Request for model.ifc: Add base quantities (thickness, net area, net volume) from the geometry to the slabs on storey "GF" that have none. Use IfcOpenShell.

First a look at what the model holds.

```python
import ifcopenshell
import ifcopenshell.util.element
import ifcopenshell.util.unit

model = ifcopenshell.open("model.ifc")
print(model.schema)
for unit_type in ("LENGTHUNIT", "AREAUNIT", "VOLUMEUNIT"):
    print(unit_type, ifcopenshell.util.unit.calculate_unit_scale(model, unit_type))
storey = next(s for s in model.by_type("IfcBuildingStorey") if s.Name == "GF")
slabs = [e for e in ifcopenshell.util.element.get_decomposition(storey) if e.is_a("IfcSlab")]
for e in sorted(slabs, key=lambda e: e.id()):
    print(e.id(), e.is_a(), e.Name, list(ifcopenshell.util.element.get_psets(e, qtos_only=True)), sep=" | ")
```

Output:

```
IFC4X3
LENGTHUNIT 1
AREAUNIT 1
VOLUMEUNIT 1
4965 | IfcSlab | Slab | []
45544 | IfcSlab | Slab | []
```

```python
import ifcopenshell
import ifcopenshell.api.pset
import ifcopenshell.geom
import ifcopenshell.util.element
import ifcopenshell.util.shape
import ifcopenshell.util.unit

model = ifcopenshell.open("model.ifc")
unit_scale = ifcopenshell.util.unit.calculate_unit_scale(model)
area_scale = ifcopenshell.util.unit.calculate_unit_scale(model, "AREAUNIT")
volume_scale = ifcopenshell.util.unit.calculate_unit_scale(model, "VOLUMEUNIT")
settings = ifcopenshell.geom.settings()

storey = next(s for s in model.by_type("IfcBuildingStorey") if s.Name == "GF")
slabs = [e for e in ifcopenshell.util.element.get_decomposition(storey) if e.is_a("IfcSlab")]

for e in sorted(slabs, key=lambda e: e.id()):
    if ifcopenshell.util.element.get_psets(e, qtos_only=True, should_inherit=False):
        continue
    # Geometry comes back in metres, in the element's own axes.
    shape = ifcopenshell.geom.create_shape(settings, e)
    values = {
        "Width": ifcopenshell.util.shape.get_z(shape.geometry) / unit_scale,
        "NetArea": ifcopenshell.util.shape.get_footprint_area(shape.geometry) / area_scale,
        "NetVolume": ifcopenshell.util.shape.get_volume(shape.geometry) / volume_scale,
    }
    qto = ifcopenshell.api.pset.add_qto(model, product=e, name="Qto_SlabBaseQuantities")
    ifcopenshell.api.pset.edit_qto(model, qto=qto, properties=values)
    print(e.id(), {k: round(v, 3) for k, v in values.items()})

model.write("model-out.ifc")
```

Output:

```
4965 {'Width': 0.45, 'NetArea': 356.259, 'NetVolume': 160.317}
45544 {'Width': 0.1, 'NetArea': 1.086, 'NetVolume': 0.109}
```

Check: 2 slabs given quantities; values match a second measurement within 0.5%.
